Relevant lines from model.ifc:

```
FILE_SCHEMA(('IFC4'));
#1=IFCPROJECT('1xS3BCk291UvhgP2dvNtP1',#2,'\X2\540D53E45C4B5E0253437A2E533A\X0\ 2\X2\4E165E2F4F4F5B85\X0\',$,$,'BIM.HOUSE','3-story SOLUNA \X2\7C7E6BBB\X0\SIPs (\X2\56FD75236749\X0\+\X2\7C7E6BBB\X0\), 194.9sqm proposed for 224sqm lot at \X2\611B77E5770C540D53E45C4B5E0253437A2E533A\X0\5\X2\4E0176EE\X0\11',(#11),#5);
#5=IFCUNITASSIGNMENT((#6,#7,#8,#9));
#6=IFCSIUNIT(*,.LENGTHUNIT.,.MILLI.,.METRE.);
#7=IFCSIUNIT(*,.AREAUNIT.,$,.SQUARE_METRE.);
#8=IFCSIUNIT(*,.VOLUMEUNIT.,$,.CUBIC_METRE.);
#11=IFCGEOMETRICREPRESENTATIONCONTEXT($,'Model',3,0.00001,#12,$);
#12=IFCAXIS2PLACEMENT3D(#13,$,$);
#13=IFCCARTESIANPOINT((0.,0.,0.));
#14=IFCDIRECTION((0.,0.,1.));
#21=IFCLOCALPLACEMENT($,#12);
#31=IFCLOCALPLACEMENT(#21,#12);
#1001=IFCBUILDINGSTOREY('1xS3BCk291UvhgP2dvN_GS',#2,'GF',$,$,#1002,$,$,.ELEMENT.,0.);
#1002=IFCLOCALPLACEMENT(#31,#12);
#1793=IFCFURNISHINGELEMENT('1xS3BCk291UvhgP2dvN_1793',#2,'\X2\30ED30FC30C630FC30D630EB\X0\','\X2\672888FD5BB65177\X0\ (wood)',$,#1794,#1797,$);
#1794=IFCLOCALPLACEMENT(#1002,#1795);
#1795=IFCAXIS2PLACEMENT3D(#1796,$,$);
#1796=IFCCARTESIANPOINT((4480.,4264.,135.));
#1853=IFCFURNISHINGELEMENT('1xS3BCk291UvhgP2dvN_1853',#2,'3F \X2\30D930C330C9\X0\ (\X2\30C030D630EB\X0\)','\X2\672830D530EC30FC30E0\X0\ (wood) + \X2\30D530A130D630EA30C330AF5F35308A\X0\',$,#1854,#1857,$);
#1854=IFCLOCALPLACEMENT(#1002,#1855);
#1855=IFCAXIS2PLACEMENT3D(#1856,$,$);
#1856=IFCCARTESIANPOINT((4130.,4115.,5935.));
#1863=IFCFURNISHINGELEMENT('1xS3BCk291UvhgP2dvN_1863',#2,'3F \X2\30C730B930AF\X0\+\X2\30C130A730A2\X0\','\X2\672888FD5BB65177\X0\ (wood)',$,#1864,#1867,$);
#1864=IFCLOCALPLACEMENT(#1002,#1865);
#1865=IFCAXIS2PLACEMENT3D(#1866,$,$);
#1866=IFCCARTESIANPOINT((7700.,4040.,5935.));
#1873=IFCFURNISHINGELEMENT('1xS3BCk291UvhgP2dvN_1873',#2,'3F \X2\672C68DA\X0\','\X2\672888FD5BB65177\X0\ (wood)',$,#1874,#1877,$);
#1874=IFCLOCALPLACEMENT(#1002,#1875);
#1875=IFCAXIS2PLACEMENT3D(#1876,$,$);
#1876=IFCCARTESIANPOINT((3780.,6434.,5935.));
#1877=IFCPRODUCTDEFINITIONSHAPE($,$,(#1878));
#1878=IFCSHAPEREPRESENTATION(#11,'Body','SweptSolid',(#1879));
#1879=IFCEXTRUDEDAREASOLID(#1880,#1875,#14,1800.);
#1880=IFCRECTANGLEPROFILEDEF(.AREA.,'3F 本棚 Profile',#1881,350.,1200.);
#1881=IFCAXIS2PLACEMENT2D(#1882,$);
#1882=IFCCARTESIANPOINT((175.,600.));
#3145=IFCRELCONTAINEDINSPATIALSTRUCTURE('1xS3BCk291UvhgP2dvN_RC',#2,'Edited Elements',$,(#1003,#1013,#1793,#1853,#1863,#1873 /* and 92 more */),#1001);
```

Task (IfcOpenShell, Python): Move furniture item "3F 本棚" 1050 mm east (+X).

```python
import ifcopenshell
import ifcopenshell.api.geometry
import ifcopenshell.util.placement

model = ifcopenshell.open("model.ifc")

item = model.by_guid("1xS3BCk291UvhgP2dvN_1873")
matrix = ifcopenshell.util.placement.get_local_placement(item.ObjectPlacement)
matrix[0, 3] += 1050.0
ifcopenshell.api.geometry.edit_object_placement(model, product=item, matrix=matrix, is_si=False)

print(ifcopenshell.util.placement.get_local_placement(item.ObjectPlacement).round(3) + 0.0)

model.write("model_edited.ifc")
```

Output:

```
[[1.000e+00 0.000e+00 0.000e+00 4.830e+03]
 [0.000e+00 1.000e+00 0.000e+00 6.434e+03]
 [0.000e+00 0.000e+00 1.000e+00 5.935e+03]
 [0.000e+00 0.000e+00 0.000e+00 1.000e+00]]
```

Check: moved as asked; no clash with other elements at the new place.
